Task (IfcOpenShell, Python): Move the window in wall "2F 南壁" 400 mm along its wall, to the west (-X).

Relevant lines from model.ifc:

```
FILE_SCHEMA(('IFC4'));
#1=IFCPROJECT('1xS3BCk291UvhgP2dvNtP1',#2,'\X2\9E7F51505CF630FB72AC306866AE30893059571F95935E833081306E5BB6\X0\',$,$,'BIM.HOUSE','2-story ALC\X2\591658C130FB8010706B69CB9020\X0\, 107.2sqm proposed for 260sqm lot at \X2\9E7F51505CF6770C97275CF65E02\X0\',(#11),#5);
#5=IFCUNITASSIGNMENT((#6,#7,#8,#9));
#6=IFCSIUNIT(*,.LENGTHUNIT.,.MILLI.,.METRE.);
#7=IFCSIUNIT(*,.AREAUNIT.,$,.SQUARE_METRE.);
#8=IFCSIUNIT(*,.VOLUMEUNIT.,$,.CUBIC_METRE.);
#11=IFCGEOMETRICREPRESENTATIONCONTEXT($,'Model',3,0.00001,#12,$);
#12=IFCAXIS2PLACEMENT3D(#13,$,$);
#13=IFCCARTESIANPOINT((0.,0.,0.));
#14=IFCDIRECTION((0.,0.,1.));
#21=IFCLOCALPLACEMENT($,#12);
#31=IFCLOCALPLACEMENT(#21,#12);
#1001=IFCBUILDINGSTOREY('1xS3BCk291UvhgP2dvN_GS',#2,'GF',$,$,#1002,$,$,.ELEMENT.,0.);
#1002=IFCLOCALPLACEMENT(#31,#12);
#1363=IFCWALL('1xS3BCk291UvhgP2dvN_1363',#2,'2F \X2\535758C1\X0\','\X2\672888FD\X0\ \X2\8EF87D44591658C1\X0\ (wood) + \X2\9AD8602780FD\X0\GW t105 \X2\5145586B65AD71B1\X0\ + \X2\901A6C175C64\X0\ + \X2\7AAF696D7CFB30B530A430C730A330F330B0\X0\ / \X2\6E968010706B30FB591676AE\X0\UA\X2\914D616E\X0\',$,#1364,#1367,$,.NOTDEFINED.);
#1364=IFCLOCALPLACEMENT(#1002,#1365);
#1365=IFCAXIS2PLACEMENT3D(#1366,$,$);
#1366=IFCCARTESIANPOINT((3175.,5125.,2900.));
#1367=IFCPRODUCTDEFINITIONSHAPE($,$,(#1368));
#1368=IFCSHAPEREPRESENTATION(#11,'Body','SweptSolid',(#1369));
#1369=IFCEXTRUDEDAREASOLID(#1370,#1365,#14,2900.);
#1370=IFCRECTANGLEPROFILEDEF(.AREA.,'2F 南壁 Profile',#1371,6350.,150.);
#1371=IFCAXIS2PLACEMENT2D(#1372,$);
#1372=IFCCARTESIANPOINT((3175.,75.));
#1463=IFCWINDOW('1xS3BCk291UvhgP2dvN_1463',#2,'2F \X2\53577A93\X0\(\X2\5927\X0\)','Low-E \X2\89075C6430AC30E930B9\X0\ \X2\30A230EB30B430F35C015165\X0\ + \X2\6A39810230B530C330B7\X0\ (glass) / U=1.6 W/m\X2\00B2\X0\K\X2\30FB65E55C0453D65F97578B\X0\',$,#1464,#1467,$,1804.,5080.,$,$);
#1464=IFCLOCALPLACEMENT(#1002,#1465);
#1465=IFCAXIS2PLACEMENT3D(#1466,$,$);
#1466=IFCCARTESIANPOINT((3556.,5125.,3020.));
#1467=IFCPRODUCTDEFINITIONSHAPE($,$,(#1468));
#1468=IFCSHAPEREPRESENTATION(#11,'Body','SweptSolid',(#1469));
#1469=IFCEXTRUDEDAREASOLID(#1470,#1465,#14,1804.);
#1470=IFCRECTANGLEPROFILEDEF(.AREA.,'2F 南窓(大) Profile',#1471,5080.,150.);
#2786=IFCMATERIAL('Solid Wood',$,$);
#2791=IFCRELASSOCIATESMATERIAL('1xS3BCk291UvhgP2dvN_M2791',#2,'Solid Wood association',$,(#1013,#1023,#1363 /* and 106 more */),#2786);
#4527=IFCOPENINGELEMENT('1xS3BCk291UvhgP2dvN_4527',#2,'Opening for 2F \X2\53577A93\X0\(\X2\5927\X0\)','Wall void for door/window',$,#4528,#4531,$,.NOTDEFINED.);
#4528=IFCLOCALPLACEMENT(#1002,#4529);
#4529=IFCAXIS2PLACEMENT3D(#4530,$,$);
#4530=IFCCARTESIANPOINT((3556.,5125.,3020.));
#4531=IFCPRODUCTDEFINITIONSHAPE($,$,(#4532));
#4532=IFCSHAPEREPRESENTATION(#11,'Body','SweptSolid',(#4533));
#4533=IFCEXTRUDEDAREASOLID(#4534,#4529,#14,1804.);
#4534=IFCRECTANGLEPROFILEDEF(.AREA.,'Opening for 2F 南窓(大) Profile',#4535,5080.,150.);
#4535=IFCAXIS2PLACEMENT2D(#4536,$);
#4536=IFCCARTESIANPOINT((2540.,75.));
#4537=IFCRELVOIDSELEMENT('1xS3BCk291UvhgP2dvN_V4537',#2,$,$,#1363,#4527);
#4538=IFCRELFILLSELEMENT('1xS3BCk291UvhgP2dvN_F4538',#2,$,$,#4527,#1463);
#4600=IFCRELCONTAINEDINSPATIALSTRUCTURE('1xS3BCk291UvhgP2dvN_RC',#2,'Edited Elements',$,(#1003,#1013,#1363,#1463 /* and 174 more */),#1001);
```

```python
import ifcopenshell
import ifcopenshell.api.geometry
import ifcopenshell.util.placement
import ifcopenshell.util.unit

model = ifcopenshell.open("model.ifc")
unit_scale = ifcopenshell.util.unit.calculate_unit_scale(model)

window = model.by_guid("1xS3BCk291UvhgP2dvN_1463")
opening = window.FillsVoids[0].RelatingOpeningElement
wall = opening.VoidsElements[0].RelatingBuildingElement

wall_matrix = ifcopenshell.util.placement.get_local_placement(wall.ObjectPlacement)
shift = wall_matrix[:3, 0] * -0.4 / unit_scale
before = ifcopenshell.util.placement.get_local_placement(window.ObjectPlacement)[:3, 3].copy()

# The window is not placed relative to its opening, so move both.
for product in (opening, window):
    matrix = ifcopenshell.util.placement.get_local_placement(product.ObjectPlacement)
    matrix[:3, 3] += shift
    ifcopenshell.api.geometry.edit_object_placement(model, product=product, matrix=matrix, is_si=False)

after = ifcopenshell.util.placement.get_local_placement(window.ObjectPlacement)[:3, 3]
print("window moved by", (after - before).round(3) + 0.0)

model.write("model_updated.ifc")
```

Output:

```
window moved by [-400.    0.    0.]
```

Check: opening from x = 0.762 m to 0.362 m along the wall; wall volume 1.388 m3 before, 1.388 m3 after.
